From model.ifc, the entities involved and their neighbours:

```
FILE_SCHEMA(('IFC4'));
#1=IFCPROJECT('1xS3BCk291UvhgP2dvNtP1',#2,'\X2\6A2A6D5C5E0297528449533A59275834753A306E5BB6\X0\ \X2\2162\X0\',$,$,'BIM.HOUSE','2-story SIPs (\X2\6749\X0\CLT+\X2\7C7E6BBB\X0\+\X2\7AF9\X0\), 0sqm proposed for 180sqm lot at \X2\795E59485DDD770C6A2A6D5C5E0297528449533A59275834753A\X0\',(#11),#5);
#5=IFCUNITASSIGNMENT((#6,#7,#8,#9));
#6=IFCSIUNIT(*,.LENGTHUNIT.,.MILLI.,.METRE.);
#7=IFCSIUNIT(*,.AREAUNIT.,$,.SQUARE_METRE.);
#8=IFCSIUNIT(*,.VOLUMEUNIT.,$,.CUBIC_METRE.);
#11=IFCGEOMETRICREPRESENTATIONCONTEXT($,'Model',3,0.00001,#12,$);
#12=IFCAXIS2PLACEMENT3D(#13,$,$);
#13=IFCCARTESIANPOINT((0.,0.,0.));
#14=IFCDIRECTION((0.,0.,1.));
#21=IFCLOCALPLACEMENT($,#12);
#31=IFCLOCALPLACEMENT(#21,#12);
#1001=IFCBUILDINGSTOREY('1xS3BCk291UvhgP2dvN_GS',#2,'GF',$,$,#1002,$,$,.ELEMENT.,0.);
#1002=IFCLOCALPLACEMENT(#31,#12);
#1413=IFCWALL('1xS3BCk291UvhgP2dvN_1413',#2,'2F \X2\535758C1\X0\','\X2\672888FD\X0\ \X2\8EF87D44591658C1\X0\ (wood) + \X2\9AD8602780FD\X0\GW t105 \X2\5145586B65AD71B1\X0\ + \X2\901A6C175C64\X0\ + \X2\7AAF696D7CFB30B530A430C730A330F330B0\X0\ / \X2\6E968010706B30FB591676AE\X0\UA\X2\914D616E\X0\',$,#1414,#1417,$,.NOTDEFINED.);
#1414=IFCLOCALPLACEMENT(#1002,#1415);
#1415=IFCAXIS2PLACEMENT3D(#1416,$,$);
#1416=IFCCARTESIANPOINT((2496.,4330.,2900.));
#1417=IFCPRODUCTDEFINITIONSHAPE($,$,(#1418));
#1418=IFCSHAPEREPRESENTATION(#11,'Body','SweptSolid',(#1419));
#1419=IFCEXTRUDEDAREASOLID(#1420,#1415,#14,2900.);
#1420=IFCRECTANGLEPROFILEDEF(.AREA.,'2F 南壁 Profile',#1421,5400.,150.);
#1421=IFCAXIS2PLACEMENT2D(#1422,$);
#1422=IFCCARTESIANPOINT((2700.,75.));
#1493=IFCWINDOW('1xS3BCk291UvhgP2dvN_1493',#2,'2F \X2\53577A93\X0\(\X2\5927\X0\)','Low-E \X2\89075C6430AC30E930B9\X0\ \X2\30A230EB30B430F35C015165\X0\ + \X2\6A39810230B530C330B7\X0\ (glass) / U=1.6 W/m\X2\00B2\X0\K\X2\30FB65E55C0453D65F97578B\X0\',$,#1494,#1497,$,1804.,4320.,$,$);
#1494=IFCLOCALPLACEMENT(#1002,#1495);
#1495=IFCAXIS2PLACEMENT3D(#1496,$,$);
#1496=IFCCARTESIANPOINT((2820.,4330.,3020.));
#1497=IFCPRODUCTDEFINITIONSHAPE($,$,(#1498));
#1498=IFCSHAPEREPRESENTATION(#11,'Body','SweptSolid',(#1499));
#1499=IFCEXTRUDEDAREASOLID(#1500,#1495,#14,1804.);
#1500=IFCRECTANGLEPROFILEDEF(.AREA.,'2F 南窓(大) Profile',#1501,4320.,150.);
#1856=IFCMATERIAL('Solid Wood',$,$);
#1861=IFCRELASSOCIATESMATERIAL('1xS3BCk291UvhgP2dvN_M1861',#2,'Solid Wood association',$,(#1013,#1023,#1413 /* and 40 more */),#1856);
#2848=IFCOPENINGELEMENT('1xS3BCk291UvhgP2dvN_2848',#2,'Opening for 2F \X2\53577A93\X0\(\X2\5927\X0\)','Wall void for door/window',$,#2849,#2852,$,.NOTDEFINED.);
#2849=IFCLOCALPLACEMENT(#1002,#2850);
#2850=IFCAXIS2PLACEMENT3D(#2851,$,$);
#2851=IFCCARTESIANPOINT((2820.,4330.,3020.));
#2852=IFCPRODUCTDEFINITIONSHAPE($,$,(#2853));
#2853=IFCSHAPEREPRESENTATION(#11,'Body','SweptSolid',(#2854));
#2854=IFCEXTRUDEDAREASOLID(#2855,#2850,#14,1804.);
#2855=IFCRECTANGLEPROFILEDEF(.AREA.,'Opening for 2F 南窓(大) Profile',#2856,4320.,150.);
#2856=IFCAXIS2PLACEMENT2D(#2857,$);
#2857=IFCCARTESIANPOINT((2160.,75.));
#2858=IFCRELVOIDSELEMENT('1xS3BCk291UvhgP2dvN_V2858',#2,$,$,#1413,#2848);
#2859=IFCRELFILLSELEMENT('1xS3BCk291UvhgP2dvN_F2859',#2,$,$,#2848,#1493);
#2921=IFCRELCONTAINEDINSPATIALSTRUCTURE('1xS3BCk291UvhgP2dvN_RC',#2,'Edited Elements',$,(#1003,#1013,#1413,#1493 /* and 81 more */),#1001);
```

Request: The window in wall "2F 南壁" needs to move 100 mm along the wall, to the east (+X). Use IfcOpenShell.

```python
import ifcopenshell
import ifcopenshell.api.geometry
import ifcopenshell.util.placement

model = ifcopenshell.open("model.ifc")

window = model.by_guid("1xS3BCk291UvhgP2dvN_1493")
opening = window.FillsVoids[0].RelatingOpeningElement
wall = opening.VoidsElements[0].RelatingBuildingElement

wall_matrix = ifcopenshell.util.placement.get_local_placement(wall.ObjectPlacement)
shift = wall_matrix[:3, 0] * 100.0
before = ifcopenshell.util.placement.get_local_placement(window.ObjectPlacement)[:3, 3].copy()

# The window is not placed relative to its opening, so move both.
for product in (opening, window):
    matrix = ifcopenshell.util.placement.get_local_placement(product.ObjectPlacement)
    matrix[:3, 3] += shift
    ifcopenshell.api.geometry.edit_object_placement(model, product=product, matrix=matrix, is_si=False)

after = ifcopenshell.util.placement.get_local_placement(window.ObjectPlacement)[:3, 3]
print("window moved by", (after - before).round(3) + 0.0)

model.write("model-out.ifc")
```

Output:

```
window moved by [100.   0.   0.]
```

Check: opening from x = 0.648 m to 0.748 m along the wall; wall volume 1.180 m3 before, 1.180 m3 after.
